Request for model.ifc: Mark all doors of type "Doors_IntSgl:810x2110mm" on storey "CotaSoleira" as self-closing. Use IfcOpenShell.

First a look at what the model holds.

```python
import ifcopenshell
import ifcopenshell.util.element

model = ifcopenshell.open("model.ifc")
print(model.schema)
storey = next(s for s in model.by_type("IfcBuildingStorey") if s.Name == "CotaSoleira")
doors = [e for e in ifcopenshell.util.element.get_decomposition(storey) if e.is_a("IfcDoor")]
seen = {}
for e in doors:
    element_type = ifcopenshell.util.element.get_type(e)
    key = (element_type.Name if element_type != e and element_type else None, ifcopenshell.util.element.get_pset(e, "Pset_DoorCommon", "SelfClosing"))
    seen[key] = seen.get(key, 0) + 1
for (name, value), count in sorted(seen.items(), key=str):
    print(count, "x", name, "|", value)
```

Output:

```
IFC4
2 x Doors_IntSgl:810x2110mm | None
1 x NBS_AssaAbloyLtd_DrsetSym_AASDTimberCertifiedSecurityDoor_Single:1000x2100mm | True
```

```python
import ifcopenshell
import ifcopenshell.api.pset
import ifcopenshell.util.element

model = ifcopenshell.open("model.ifc")

storey = next(s for s in model.by_type("IfcBuildingStorey") if s.Name == "CotaSoleira")
doors = [e for e in ifcopenshell.util.element.get_decomposition(storey) if e.is_a("IfcDoor")]

count = 0
for e in doors:
    element_type = ifcopenshell.util.element.get_type(e)
    if element_type in (None, e) or element_type.Name != "Doors_IntSgl:810x2110mm":
        continue
    # add_pset returns the element's existing set when there is one.
    pset = ifcopenshell.api.pset.add_pset(model, product=e, name="Pset_DoorCommon")
    ifcopenshell.api.pset.edit_pset(model, pset=pset, properties={"SelfClosing": True})
    count += 1

print(count, "doors updated")

model.write("model-out.ifc")
```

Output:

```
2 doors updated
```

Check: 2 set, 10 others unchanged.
